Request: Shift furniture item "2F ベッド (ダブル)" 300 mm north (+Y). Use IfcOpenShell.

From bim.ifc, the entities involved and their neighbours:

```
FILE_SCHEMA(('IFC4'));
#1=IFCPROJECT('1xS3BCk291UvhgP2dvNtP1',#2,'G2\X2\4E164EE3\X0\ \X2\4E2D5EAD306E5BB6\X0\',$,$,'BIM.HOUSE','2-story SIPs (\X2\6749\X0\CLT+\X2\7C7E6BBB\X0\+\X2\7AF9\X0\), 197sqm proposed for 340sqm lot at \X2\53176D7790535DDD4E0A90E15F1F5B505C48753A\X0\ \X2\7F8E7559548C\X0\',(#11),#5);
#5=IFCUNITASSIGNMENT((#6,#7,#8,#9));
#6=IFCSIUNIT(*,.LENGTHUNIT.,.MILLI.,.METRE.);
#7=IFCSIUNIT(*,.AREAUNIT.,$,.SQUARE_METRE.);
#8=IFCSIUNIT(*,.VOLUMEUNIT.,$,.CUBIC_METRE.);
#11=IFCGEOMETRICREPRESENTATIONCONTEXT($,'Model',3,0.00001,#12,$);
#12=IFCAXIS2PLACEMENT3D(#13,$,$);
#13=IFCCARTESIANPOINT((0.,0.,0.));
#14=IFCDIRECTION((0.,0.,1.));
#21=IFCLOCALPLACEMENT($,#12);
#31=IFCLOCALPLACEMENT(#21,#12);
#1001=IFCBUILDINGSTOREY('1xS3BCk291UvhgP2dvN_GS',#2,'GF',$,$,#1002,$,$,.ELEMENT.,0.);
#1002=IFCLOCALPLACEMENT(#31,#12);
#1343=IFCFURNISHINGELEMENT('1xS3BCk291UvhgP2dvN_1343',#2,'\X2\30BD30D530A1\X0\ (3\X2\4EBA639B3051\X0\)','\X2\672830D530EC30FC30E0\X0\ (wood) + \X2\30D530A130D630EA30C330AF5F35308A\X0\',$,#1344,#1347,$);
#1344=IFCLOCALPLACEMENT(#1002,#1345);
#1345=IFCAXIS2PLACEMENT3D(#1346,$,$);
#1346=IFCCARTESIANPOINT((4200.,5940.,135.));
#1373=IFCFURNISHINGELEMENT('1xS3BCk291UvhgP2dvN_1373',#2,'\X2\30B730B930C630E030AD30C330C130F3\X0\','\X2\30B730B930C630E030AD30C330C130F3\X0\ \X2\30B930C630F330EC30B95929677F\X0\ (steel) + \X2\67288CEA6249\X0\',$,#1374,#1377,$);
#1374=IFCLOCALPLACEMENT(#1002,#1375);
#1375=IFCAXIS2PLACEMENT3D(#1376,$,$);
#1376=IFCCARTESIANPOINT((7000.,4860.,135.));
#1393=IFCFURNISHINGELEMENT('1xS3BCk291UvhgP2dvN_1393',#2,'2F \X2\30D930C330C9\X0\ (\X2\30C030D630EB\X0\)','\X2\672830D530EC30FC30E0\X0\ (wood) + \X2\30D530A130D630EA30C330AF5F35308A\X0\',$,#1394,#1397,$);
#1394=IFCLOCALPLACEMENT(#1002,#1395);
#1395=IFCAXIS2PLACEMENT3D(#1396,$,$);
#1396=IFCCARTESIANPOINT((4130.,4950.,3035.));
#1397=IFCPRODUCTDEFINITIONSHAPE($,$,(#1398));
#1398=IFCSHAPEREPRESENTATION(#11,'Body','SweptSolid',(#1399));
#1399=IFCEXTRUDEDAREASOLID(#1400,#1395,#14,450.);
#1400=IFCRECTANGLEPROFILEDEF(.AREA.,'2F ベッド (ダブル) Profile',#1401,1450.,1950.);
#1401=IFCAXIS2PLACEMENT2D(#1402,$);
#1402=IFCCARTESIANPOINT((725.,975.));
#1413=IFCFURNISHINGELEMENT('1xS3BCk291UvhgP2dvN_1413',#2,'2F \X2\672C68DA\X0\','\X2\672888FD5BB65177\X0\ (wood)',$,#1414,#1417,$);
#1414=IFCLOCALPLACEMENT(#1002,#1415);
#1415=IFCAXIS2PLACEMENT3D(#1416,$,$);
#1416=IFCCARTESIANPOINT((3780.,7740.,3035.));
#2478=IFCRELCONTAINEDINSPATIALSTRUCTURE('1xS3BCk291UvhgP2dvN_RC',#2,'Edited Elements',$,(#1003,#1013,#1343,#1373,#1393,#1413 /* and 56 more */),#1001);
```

```python
import ifcopenshell
import ifcopenshell.api.geometry
import ifcopenshell.util.placement

model = ifcopenshell.open("bim.ifc")

item = model.by_guid("1xS3BCk291UvhgP2dvN_1393")
matrix = ifcopenshell.util.placement.get_local_placement(item.ObjectPlacement)
matrix[1, 3] += 300.0
ifcopenshell.api.geometry.edit_object_placement(model, product=item, matrix=matrix, is_si=False)

print(ifcopenshell.util.placement.get_local_placement(item.ObjectPlacement).round(3) + 0.0)

model.write("bim_rev.ifc")
```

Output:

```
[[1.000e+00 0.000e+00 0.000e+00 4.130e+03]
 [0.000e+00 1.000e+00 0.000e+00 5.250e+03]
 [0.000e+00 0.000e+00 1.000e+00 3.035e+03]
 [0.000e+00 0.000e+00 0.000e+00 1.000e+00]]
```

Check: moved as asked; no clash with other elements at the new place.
